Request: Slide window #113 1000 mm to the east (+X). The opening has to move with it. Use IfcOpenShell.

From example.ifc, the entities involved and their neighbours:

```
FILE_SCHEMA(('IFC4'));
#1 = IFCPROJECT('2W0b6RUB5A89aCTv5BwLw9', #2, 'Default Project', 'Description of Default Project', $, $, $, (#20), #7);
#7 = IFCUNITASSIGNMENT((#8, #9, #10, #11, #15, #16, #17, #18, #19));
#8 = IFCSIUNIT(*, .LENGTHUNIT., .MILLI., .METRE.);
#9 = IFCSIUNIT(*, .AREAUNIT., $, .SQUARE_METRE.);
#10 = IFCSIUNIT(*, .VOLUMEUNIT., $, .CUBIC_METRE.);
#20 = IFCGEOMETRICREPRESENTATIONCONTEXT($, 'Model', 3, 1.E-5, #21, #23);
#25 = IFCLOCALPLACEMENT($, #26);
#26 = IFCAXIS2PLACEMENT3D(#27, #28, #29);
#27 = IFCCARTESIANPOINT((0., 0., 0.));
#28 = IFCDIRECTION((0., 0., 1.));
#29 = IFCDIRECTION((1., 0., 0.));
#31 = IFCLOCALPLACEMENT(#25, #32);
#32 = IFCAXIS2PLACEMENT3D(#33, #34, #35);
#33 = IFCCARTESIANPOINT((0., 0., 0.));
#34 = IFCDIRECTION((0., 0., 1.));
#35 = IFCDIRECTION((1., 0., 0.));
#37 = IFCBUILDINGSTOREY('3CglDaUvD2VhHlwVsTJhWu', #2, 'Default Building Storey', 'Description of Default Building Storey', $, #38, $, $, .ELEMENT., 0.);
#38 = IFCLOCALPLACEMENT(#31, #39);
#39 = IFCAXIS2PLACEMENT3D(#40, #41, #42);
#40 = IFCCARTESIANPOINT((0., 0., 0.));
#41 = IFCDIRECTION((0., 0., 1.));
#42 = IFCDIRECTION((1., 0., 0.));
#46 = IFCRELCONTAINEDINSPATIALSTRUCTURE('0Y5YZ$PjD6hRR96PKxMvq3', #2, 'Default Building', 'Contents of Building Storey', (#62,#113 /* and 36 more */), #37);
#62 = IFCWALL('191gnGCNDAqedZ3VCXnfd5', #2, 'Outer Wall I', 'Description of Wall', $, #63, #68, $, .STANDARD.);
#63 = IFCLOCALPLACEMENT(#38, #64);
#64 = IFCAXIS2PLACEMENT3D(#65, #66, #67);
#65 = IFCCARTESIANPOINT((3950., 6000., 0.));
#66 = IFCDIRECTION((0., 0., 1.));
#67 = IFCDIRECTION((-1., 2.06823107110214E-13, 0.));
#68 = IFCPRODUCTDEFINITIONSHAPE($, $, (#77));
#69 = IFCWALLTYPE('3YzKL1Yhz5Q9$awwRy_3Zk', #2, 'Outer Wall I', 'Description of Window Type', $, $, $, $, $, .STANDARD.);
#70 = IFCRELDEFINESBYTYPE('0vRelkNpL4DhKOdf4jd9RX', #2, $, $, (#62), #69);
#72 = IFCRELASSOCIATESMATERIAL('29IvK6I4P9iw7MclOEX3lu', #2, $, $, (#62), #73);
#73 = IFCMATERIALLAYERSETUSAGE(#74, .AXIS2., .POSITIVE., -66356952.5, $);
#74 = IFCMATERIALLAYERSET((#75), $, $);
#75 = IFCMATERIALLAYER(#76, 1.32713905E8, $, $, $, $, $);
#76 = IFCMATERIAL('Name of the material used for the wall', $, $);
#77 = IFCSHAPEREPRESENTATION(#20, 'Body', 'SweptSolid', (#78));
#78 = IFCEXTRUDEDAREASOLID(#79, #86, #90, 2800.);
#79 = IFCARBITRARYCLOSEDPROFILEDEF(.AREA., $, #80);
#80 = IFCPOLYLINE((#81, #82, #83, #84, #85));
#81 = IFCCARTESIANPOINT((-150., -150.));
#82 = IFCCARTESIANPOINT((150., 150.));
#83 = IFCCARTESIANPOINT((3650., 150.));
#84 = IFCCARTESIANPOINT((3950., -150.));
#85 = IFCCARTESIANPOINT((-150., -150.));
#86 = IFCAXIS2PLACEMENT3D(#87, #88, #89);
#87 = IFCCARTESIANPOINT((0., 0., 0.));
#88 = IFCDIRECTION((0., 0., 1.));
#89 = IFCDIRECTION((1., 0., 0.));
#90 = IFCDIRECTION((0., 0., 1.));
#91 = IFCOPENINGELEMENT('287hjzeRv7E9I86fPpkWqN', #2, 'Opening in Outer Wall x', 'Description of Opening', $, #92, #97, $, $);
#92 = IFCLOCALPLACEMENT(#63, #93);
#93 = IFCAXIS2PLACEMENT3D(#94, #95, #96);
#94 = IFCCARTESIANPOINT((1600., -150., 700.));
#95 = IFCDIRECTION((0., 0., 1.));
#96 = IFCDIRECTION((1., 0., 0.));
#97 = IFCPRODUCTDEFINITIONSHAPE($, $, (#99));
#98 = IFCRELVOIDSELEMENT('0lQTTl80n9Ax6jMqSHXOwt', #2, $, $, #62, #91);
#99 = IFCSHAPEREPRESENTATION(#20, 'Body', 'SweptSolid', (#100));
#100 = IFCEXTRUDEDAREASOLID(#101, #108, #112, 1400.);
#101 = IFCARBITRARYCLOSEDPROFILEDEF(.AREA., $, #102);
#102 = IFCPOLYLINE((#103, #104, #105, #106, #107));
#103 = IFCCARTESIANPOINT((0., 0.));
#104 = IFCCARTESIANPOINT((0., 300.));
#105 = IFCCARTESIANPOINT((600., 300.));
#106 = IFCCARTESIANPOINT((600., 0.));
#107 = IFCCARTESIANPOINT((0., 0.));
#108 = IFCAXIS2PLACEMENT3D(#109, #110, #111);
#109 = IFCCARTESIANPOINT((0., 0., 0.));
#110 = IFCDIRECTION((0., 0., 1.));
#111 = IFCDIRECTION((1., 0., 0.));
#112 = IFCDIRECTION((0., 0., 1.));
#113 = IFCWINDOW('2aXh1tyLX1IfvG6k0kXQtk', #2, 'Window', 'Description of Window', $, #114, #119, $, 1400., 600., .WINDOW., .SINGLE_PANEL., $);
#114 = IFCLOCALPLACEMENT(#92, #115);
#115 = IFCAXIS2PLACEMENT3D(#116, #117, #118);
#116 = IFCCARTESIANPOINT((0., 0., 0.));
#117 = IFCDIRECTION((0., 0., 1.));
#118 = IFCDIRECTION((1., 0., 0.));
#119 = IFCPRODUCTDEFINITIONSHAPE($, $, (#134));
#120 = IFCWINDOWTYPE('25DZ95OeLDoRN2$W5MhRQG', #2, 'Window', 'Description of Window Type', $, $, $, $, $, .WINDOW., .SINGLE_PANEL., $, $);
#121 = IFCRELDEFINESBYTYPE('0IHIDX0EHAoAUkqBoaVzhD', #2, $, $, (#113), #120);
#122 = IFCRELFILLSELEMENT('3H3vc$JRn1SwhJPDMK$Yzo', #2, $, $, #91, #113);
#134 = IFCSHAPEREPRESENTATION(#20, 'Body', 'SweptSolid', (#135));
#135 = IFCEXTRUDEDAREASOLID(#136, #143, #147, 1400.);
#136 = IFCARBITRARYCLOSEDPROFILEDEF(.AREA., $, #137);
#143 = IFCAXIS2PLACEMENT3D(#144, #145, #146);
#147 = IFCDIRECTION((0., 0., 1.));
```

```python
import ifcopenshell
import ifcopenshell.api.geometry
import ifcopenshell.util.placement
import ifcopenshell.util.unit

model = ifcopenshell.open("example.ifc")
unit_scale = ifcopenshell.util.unit.calculate_unit_scale(model)

window = model.by_guid("2aXh1tyLX1IfvG6k0kXQtk")
opening = window.FillsVoids[0].RelatingOpeningElement
wall = opening.VoidsElements[0].RelatingBuildingElement

wall_matrix = ifcopenshell.util.placement.get_local_placement(wall.ObjectPlacement)
shift = wall_matrix[:3, 0] * -1 / unit_scale
before = ifcopenshell.util.placement.get_local_placement(window.ObjectPlacement)[:3, 3].copy()

# The window is placed relative to its opening, so it follows when the opening moves.
matrix = ifcopenshell.util.placement.get_local_placement(opening.ObjectPlacement)
matrix[:3, 3] += shift
ifcopenshell.api.geometry.edit_object_placement(
    model, product=opening, matrix=matrix, is_si=False, should_transform_children=True
)

after = ifcopenshell.util.placement.get_local_placement(window.ObjectPlacement)[:3, 3]
print("window moved by", (after - before).round(3) + 0.0)

model.write("example_v2.ifc")
```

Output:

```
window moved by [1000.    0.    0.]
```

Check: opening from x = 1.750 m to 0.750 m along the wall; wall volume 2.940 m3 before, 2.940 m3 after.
